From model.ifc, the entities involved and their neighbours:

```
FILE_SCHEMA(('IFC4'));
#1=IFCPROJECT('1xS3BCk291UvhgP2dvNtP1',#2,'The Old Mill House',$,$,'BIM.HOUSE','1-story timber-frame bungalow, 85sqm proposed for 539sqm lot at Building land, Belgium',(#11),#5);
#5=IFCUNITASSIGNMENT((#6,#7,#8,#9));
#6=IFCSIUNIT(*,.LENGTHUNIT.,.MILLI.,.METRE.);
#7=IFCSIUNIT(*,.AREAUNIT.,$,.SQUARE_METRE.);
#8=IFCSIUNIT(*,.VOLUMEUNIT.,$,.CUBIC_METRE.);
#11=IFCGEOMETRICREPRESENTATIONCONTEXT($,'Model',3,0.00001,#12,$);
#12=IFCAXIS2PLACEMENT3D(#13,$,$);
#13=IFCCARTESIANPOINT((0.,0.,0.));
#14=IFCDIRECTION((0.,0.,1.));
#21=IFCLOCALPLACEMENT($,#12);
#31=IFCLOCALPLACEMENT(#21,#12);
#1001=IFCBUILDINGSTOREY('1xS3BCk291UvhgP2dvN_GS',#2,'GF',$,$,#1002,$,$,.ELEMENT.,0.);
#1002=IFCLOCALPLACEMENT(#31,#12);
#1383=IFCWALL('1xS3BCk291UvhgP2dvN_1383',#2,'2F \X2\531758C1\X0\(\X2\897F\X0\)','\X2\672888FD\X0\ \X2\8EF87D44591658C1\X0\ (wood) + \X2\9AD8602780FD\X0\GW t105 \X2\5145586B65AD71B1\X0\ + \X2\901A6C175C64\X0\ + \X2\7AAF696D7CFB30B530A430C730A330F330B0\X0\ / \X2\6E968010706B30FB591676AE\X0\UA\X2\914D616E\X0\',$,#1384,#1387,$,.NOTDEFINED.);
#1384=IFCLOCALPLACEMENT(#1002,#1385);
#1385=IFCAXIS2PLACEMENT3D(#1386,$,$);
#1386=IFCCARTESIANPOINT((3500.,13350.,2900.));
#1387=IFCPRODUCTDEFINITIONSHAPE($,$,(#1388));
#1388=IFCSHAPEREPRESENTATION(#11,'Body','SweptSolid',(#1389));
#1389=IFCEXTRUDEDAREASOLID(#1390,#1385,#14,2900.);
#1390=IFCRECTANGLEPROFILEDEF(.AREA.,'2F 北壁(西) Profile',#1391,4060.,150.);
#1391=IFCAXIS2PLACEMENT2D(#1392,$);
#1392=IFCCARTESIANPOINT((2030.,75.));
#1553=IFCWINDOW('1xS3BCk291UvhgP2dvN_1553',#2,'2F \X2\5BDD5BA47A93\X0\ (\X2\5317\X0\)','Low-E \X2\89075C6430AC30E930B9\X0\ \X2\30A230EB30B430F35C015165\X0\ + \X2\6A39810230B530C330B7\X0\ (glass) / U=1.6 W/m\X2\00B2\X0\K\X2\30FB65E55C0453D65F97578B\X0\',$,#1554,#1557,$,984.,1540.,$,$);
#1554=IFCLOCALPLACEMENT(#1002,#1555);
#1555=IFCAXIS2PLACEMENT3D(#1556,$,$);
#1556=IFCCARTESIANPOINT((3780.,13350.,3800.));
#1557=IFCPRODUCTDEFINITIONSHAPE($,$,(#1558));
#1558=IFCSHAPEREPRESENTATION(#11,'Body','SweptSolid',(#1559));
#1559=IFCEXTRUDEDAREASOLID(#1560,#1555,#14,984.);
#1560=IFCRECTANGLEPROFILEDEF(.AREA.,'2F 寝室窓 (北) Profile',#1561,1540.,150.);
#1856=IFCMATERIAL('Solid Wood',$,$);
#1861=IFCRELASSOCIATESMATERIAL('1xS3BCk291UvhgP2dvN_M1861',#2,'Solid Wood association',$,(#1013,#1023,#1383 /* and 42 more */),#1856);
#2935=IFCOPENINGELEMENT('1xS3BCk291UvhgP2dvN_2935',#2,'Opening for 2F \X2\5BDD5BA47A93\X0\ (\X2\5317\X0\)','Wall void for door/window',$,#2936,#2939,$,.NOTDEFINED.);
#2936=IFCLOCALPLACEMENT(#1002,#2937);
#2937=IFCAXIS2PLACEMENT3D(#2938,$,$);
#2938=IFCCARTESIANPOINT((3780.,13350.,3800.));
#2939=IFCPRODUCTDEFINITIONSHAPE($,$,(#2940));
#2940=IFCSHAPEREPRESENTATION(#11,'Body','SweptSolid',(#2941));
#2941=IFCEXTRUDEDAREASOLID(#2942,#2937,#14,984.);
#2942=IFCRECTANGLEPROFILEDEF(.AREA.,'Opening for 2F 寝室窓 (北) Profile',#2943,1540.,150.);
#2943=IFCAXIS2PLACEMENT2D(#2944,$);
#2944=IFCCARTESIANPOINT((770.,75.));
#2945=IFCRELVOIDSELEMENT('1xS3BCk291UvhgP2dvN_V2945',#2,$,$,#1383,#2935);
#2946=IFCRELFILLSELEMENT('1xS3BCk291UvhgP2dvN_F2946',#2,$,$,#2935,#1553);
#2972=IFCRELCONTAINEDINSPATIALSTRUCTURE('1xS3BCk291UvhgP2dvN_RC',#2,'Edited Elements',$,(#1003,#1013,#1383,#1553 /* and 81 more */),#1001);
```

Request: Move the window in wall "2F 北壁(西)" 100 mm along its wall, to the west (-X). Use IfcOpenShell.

```python
import ifcopenshell
import ifcopenshell.api.geometry
import ifcopenshell.util.placement
import ifcopenshell.util.unit

model = ifcopenshell.open("model.ifc")
unit_scale = ifcopenshell.util.unit.calculate_unit_scale(model)

window = model.by_id(1553)
opening = window.FillsVoids[0].RelatingOpeningElement
wall = opening.VoidsElements[0].RelatingBuildingElement

wall_matrix = ifcopenshell.util.placement.get_local_placement(wall.ObjectPlacement)
shift = wall_matrix[:3, 0] * -0.1 / unit_scale
before = ifcopenshell.util.placement.get_local_placement(window.ObjectPlacement)[:3, 3].copy()

# The window is not placed relative to its opening, so move both.
for product in (opening, window):
    matrix = ifcopenshell.util.placement.get_local_placement(product.ObjectPlacement)
    matrix[:3, 3] += shift
    ifcopenshell.api.geometry.edit_object_placement(model, product=product, matrix=matrix, is_si=False)

after = ifcopenshell.util.placement.get_local_placement(window.ObjectPlacement)[:3, 3]
print("window moved by", (after - before).round(3) + 0.0)

model.write("model_rev.ifc")
```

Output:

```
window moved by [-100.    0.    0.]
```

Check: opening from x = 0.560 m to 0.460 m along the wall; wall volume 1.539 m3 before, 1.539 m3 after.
